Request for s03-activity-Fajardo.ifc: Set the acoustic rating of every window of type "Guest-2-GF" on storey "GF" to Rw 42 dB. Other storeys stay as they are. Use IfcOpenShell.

First a look at what the model holds.

```python
import ifcopenshell
import ifcopenshell.util.element

model = ifcopenshell.open("s03-activity-Fajardo.ifc")
print(model.schema)
storey = next(s for s in model.by_type("IfcBuildingStorey") if s.Name == "GF")
windows = [e for e in ifcopenshell.util.element.get_decomposition(storey) if e.is_a("IfcWindow")]
seen = {}
for e in windows:
    element_type = ifcopenshell.util.element.get_type(e)
    key = (element_type.Name if element_type != e and element_type else None, ifcopenshell.util.element.get_pset(e, "Pset_WindowCommon", "AcousticRating"))
    seen[key] = seen.get(key, 0) + 1
for (name, value), count in sorted(seen.items(), key=str):
    print(count, "x", name, "|", value)
```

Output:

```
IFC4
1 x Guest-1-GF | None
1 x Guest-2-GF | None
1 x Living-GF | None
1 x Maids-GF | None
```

```python
import ifcopenshell
import ifcopenshell.api.pset
import ifcopenshell.util.element

model = ifcopenshell.open("s03-activity-Fajardo.ifc")

storey = next(s for s in model.by_type("IfcBuildingStorey") if s.Name == "GF")
windows = [e for e in ifcopenshell.util.element.get_decomposition(storey) if e.is_a("IfcWindow")]

count = 0
for e in windows:
    element_type = ifcopenshell.util.element.get_type(e)
    if element_type in (None, e) or element_type.Name != "Guest-2-GF":
        continue
    # add_pset returns the element's existing set when there is one.
    pset = ifcopenshell.api.pset.add_pset(model, product=e, name="Pset_WindowCommon")
    ifcopenshell.api.pset.edit_pset(model, pset=pset, properties={"AcousticRating": "Rw 42 dB"})
    count += 1

print(count, "windows updated")

model.write("s03-activity-Fajardo-out.ifc")
```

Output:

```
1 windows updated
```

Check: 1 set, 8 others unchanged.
